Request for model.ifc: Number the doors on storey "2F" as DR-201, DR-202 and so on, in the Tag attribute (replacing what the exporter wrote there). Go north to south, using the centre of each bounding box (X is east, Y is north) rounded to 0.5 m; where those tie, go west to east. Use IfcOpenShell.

First a look at what the model holds.

```python
import ifcopenshell
import ifcopenshell.util.element
import ifcopenshell.util.placement

model = ifcopenshell.open("model.ifc")
print(model.schema)
storey = next(s for s in model.by_type("IfcBuildingStorey") if s.Name == "2F")
doors = [e for e in ifcopenshell.util.element.get_decomposition(storey) if e.is_a("IfcDoor")]
for e in sorted(doors, key=lambda e: e.id()):
    origin = ifcopenshell.util.placement.get_local_placement(e.ObjectPlacement)[:3, 3]
    print(e.id(), e.Tag, e.Name, origin.round(2) + 0.0, sep=" | ")
```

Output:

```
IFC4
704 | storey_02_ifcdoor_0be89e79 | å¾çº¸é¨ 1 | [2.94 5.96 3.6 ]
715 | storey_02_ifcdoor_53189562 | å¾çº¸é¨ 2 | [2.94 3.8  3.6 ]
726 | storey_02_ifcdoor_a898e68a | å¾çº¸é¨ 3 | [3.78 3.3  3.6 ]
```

```python
import ifcopenshell
import ifcopenshell.geom
import ifcopenshell.util.element
import ifcopenshell.util.shape

model = ifcopenshell.open("model.ifc")
settings = ifcopenshell.geom.settings()
settings.set("use-world-coords", True)


def centre(element):
    shape = ifcopenshell.geom.create_shape(settings, element)
    return ifcopenshell.util.shape.get_bbox_centroid(shape.geometry)


storey = next(s for s in model.by_type("IfcBuildingStorey") if s.Name == "2F")
doors = [e for e in ifcopenshell.util.element.get_decomposition(storey) if e.is_a("IfcDoor")]

# Insertion points can sit at a corner or the storey origin, so sort by the geometry (in metres).
centres = {e: centre(e) for e in doors}
doors.sort(key=lambda e: (-round(centres[e][1] / 0.5), centres[e][0]))

for i, e in enumerate(doors, start=1):
    number = f"DR-2{i:02d}"
    e.Tag = number
    print(e.id(), number)

model.write("model_edited.ifc")
```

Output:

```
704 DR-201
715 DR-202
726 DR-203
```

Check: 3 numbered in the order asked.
